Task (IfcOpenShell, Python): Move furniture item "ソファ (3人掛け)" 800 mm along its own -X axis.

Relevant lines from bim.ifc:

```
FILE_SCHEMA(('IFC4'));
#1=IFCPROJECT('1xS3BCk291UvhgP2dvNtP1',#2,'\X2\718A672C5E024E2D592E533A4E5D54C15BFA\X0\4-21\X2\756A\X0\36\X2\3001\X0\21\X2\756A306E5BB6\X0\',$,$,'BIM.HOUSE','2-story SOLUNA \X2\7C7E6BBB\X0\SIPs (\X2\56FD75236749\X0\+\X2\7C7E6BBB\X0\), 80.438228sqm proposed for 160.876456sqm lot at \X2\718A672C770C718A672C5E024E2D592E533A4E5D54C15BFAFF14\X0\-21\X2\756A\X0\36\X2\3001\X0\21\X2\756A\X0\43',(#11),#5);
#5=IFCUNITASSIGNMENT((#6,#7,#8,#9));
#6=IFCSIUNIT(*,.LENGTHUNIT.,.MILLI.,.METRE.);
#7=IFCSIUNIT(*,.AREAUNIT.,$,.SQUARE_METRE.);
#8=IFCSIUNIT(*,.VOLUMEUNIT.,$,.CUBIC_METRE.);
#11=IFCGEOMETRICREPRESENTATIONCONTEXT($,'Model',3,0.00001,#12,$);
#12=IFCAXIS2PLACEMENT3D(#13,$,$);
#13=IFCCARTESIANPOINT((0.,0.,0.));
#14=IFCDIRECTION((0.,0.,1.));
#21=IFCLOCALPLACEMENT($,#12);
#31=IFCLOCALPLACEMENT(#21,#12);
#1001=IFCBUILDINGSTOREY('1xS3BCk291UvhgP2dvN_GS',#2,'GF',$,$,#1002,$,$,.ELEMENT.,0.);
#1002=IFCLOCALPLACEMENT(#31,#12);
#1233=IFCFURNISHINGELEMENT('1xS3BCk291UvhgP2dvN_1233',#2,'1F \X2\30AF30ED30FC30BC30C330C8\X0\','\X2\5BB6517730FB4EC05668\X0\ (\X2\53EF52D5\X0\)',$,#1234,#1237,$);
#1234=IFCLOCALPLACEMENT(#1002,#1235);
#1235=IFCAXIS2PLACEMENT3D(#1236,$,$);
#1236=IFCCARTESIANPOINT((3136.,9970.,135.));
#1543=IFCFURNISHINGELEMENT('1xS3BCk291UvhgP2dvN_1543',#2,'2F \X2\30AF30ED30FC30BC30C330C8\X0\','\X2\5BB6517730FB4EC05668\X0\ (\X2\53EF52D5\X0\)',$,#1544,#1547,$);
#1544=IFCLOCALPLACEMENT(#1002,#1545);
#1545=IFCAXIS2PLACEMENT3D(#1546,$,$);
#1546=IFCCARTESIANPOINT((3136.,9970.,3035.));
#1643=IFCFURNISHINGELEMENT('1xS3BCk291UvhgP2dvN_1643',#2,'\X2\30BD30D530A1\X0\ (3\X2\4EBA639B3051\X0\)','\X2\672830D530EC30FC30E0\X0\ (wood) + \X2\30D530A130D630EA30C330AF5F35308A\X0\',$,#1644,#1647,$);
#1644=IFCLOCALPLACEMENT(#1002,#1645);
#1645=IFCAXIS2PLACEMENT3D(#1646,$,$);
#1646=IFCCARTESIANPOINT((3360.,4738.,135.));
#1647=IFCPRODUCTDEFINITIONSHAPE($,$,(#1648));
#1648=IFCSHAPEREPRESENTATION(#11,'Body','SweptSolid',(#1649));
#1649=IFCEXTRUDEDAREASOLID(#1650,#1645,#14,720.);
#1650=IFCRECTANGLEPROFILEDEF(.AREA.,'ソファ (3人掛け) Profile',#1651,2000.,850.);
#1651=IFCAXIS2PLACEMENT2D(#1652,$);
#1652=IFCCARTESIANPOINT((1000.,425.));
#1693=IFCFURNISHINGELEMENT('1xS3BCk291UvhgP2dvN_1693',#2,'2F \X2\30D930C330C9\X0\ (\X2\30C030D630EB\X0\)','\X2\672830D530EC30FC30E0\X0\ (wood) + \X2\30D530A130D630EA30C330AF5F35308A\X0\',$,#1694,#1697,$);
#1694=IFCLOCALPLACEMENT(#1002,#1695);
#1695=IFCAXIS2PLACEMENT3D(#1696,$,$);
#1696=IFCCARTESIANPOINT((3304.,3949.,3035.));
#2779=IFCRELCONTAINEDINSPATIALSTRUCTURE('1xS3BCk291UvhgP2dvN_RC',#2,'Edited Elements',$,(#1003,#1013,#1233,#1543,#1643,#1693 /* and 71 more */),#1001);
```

```python
import ifcopenshell
import ifcopenshell.api.geometry
import ifcopenshell.util.placement
import ifcopenshell.util.unit

model = ifcopenshell.open("bim.ifc")
unit_scale = ifcopenshell.util.unit.calculate_unit_scale(model)

item = model.by_guid("1xS3BCk291UvhgP2dvN_1643")
matrix = ifcopenshell.util.placement.get_local_placement(item.ObjectPlacement)
matrix[:3, 3] -= matrix[:3, 0] * 0.8 / unit_scale
ifcopenshell.api.geometry.edit_object_placement(model, product=item, matrix=matrix, is_si=False)

print(ifcopenshell.util.placement.get_local_placement(item.ObjectPlacement).round(3) + 0.0)

model.write("bim_v2.ifc")
```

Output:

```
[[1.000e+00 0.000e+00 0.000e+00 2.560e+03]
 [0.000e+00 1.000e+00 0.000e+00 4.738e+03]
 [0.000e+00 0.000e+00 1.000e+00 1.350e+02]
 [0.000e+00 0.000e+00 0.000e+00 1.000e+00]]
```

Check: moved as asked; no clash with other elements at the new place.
